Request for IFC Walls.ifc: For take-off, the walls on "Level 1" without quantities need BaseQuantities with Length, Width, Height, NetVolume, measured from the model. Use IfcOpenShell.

First a look at what the model holds.

```python
import ifcopenshell
import ifcopenshell.util.element
import ifcopenshell.util.unit

model = ifcopenshell.open("IFC Walls.ifc")
print(model.schema)
for unit_type in ("LENGTHUNIT", "AREAUNIT", "VOLUMEUNIT"):
    print(unit_type, ifcopenshell.util.unit.calculate_unit_scale(model, unit_type))
storey = next(s for s in model.by_type("IfcBuildingStorey") if s.Name == "Level 1")
walls = [e for e in ifcopenshell.util.element.get_decomposition(storey) if e.is_a("IfcWall")]
for e in sorted(walls, key=lambda e: e.id()):
    print(e.id(), e.is_a(), e.Name, list(ifcopenshell.util.element.get_psets(e, qtos_only=True)), sep=" | ")
```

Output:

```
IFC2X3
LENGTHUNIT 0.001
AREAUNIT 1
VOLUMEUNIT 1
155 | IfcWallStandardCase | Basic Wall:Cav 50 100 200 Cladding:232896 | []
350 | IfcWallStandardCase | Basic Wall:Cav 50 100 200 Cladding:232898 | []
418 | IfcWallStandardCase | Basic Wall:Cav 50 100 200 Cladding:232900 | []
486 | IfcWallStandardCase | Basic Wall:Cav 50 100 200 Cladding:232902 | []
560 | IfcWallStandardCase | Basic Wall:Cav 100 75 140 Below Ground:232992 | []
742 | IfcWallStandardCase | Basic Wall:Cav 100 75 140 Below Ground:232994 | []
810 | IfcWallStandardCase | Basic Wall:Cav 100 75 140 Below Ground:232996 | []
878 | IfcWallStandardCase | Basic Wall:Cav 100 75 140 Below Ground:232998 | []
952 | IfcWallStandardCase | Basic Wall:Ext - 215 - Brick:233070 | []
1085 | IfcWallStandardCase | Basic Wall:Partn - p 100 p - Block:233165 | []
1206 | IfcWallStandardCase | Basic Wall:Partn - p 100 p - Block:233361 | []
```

```python
import ifcopenshell
import ifcopenshell.api.pset
import ifcopenshell.geom
import ifcopenshell.util.element
import ifcopenshell.util.shape
import ifcopenshell.util.unit

model = ifcopenshell.open("IFC Walls.ifc")
unit_scale = ifcopenshell.util.unit.calculate_unit_scale(model)
volume_scale = ifcopenshell.util.unit.calculate_unit_scale(model, "VOLUMEUNIT")
settings = ifcopenshell.geom.settings()

storey = next(s for s in model.by_type("IfcBuildingStorey") if s.Name == "Level 1")
walls = [e for e in ifcopenshell.util.element.get_decomposition(storey) if e.is_a("IfcWall")]

for e in sorted(walls, key=lambda e: e.id()):
    if ifcopenshell.util.element.get_psets(e, qtos_only=True, should_inherit=False):
        continue
    # Geometry comes back in metres, in the element's own axes.
    shape = ifcopenshell.geom.create_shape(settings, e)
    values = {
        "Length": ifcopenshell.util.shape.get_x(shape.geometry) / unit_scale,
        "Width": ifcopenshell.util.shape.get_y(shape.geometry) / unit_scale,
        "Height": ifcopenshell.util.shape.get_z(shape.geometry) / unit_scale,
        "NetVolume": ifcopenshell.util.shape.get_volume(shape.geometry) / volume_scale,
    }
    qto = ifcopenshell.api.pset.add_qto(model, product=e, name="BaseQuantities")
    ifcopenshell.api.pset.edit_qto(model, qto=qto, properties=values)
    print(e.id(), {k: round(v, 3) for k, v in values.items()})

model.write("IFC Walls_v2.ifc")
```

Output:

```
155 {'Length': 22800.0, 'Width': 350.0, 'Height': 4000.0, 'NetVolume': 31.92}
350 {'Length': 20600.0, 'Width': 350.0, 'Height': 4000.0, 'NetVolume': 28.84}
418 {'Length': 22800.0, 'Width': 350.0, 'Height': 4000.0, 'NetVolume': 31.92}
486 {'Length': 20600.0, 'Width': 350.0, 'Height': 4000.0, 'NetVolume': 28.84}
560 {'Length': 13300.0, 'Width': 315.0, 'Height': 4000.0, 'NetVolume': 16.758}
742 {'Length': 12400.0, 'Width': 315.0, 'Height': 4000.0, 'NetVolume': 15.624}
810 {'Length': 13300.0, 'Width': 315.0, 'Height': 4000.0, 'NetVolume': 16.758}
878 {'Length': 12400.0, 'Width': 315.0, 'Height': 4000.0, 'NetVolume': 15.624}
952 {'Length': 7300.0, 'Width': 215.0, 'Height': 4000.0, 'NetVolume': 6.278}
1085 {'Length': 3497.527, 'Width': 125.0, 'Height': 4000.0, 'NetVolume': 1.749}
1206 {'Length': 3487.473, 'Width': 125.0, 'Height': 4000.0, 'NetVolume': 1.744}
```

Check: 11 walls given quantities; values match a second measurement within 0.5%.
